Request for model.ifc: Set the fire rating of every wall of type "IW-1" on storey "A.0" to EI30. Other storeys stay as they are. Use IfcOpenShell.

First a look at what the model holds.

```python
import ifcopenshell
import ifcopenshell.util.element

model = ifcopenshell.open("model.ifc")
print(model.schema)
storey = next(s for s in model.by_type("IfcBuildingStorey") if s.Name == "A.0")
walls = [e for e in ifcopenshell.util.element.get_decomposition(storey) if e.is_a("IfcWall")]
seen = {}
for e in walls:
    element_type = ifcopenshell.util.element.get_type(e)
    key = (element_type.Name if element_type != e and element_type else None, ifcopenshell.util.element.get_pset(e, "Pset_WallCommon", "FireRating"))
    seen[key] = seen.get(key, 0) + 1
for (name, value), count in sorted(seen.items(), key=str):
    print(count, "x", name, "|", value)
```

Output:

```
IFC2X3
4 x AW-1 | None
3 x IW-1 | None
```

```python
import ifcopenshell
import ifcopenshell.api.pset
import ifcopenshell.util.element

model = ifcopenshell.open("model.ifc")

storey = next(s for s in model.by_type("IfcBuildingStorey") if s.Name == "A.0")
walls = [e for e in ifcopenshell.util.element.get_decomposition(storey) if e.is_a("IfcWall")]

count = 0
for e in walls:
    element_type = ifcopenshell.util.element.get_type(e)
    if element_type in (None, e) or element_type.Name != "IW-1":
        continue
    # add_pset returns the element's existing set when there is one.
    pset = ifcopenshell.api.pset.add_pset(model, product=e, name="Pset_WallCommon")
    ifcopenshell.api.pset.edit_pset(model, pset=pset, properties={"FireRating": "EI30"})
    count += 1

print(count, "walls updated")

model.write("model_v2.ifc")
```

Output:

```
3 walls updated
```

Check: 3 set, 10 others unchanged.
